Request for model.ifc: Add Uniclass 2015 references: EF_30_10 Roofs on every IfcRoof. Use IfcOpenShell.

First a look at what the model holds.

```python
import ifcopenshell

model = ifcopenshell.open("model.ifc")
print(model.schema)
print("classifications:", [c.Name for c in model.by_type("IfcClassification")])
for ifc_class in ("IfcDoor", "IfcRoof", "IfcStair", "IfcWall", "IfcWindow"):
    print(ifc_class, len(model.by_type(ifc_class)))
```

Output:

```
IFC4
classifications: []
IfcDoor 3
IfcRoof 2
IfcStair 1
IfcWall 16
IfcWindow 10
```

```python
import ifcopenshell
import ifcopenshell.api.classification

model = ifcopenshell.open("model.ifc")

system = ifcopenshell.api.classification.add_classification(model, classification="Uniclass 2015")

codes = {
    "IfcRoof": ("EF_30_10", "Roofs"),
}
for ifc_class, (code, name) in codes.items():
    products = model.by_type(ifc_class)
    ifcopenshell.api.classification.add_reference(
        model, products=products, classification=system, identification=code, name=name
    )
    print(code, len(products))

model.write("model_v2.ifc")
```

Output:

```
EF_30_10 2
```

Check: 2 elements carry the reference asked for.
